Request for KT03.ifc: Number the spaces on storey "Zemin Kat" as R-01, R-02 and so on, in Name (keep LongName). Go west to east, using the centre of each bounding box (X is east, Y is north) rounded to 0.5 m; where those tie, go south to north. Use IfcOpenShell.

First a look at what the model holds.

```python
import ifcopenshell
import ifcopenshell.util.element
import ifcopenshell.util.placement

model = ifcopenshell.open("KT03.ifc")
print(model.schema)
storey = next(s for s in model.by_type("IfcBuildingStorey") if s.Name == "Zemin Kat")
spaces = [e for e in ifcopenshell.util.element.get_decomposition(storey) if e.is_a("IfcSpace")]
for e in sorted(spaces, key=lambda e: e.id()):
    origin = ifcopenshell.util.placement.get_local_placement(e.ObjectPlacement)[:3, 3]
    print(e.id(), e.Name, e.LongName, origin.round(2) + 0.0, sep=" | ")
```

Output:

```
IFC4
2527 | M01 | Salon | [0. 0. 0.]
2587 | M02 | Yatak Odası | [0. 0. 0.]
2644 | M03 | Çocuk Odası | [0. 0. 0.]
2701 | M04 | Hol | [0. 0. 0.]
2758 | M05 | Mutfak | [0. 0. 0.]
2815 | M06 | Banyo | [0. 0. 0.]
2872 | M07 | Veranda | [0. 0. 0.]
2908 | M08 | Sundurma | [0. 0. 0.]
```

```python
import ifcopenshell
import ifcopenshell.geom
import ifcopenshell.util.element
import ifcopenshell.util.shape

model = ifcopenshell.open("KT03.ifc")
settings = ifcopenshell.geom.settings()
settings.set("use-world-coords", True)


def centre(element):
    shape = ifcopenshell.geom.create_shape(settings, element)
    return ifcopenshell.util.shape.get_bbox_centroid(shape.geometry)


storey = next(s for s in model.by_type("IfcBuildingStorey") if s.Name == "Zemin Kat")
spaces = [e for e in ifcopenshell.util.element.get_decomposition(storey) if e.is_a("IfcSpace")]

# Insertion points can sit at a corner or the storey origin, so sort by the geometry (in metres).
centres = {e: centre(e) for e in spaces}
spaces.sort(key=lambda e: (round(centres[e][0] / 0.5), centres[e][1]))

for i, e in enumerate(spaces, start=1):
    number = f"R-{i:02d}"
    e.Name = number
    print(e.id(), number)

model.write("KT03_rev.ifc")
```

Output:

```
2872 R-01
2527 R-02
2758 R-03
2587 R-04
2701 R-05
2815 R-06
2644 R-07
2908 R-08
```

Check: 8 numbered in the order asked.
